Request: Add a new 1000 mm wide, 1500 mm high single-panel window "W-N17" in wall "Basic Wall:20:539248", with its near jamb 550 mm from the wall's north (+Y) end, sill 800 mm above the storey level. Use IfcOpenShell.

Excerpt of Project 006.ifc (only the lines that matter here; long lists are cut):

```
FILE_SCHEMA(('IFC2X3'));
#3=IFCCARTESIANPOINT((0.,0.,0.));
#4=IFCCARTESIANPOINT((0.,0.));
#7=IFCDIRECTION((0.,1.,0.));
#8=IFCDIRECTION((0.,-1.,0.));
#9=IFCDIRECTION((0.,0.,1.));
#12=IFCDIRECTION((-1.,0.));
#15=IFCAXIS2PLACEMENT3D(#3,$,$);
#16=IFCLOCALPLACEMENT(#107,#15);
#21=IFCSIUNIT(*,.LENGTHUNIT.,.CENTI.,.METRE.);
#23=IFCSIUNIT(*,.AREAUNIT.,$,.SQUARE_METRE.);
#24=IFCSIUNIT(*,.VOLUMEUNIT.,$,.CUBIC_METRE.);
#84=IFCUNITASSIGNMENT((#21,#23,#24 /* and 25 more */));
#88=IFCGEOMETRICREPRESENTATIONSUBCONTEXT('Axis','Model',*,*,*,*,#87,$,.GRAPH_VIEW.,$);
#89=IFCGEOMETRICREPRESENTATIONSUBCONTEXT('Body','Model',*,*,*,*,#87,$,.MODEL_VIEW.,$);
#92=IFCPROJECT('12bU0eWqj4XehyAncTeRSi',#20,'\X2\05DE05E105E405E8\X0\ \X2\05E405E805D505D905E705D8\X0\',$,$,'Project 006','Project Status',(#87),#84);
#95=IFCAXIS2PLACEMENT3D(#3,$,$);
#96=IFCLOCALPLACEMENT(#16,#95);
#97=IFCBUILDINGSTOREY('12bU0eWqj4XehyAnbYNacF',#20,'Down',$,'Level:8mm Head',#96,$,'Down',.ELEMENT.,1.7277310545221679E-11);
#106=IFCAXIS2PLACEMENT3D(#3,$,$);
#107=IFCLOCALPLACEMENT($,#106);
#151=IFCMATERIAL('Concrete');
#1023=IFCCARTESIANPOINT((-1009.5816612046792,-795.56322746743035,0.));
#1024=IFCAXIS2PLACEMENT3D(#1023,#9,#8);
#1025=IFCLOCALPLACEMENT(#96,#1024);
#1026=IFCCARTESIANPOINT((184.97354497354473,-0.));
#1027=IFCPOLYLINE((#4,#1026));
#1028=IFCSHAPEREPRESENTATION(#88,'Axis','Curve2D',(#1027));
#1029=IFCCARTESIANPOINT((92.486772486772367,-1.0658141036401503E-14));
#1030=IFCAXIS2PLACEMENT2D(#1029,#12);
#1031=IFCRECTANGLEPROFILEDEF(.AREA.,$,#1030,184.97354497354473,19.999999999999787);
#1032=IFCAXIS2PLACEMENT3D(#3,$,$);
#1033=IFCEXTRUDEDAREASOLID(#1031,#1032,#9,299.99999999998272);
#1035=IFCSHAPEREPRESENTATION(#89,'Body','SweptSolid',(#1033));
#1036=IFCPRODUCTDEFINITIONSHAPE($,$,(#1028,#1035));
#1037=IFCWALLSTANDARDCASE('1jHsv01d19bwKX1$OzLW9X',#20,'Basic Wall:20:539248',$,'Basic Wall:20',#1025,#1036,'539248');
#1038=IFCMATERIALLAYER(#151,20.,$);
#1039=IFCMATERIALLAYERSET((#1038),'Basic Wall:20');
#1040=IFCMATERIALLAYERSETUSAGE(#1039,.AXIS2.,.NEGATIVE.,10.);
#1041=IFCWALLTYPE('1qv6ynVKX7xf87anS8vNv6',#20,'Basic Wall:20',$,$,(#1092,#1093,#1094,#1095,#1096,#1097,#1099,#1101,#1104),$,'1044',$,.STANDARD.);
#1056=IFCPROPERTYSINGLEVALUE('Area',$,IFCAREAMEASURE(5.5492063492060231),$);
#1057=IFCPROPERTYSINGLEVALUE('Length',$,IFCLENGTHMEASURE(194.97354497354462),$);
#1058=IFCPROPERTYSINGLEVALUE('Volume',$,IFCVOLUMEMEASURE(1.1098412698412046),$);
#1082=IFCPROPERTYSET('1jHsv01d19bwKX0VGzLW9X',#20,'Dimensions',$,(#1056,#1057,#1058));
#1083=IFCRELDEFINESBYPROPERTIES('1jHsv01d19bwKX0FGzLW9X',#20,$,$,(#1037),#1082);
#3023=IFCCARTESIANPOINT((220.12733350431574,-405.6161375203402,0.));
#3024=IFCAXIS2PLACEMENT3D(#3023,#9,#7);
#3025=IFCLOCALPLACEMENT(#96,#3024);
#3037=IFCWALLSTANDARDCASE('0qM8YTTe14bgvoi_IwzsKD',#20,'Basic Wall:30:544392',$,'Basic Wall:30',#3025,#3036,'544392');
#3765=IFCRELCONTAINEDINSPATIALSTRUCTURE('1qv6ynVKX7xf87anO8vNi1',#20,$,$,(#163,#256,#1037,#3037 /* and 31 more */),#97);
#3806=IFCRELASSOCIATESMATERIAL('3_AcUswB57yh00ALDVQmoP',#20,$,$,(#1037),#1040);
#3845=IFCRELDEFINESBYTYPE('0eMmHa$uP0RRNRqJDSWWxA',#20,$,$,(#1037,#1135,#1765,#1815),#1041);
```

```python
import numpy as np
import ifcopenshell
import ifcopenshell.api.feature
import ifcopenshell.api.geometry
import ifcopenshell.api.pset
import ifcopenshell.api.root
import ifcopenshell.api.spatial
import ifcopenshell.api.type
import ifcopenshell.geom
import ifcopenshell.util.element
import ifcopenshell.util.placement
import ifcopenshell.util.representation
import ifcopenshell.util.shape
import ifcopenshell.util.unit

model = ifcopenshell.open("Project 006.ifc")
unit_scale = ifcopenshell.util.unit.calculate_unit_scale(model)
area_scale = ifcopenshell.util.unit.calculate_unit_scale(model, "AREAUNIT")
volume_scale = ifcopenshell.util.unit.calculate_unit_scale(model, "VOLUMEUNIT")
settings = ifcopenshell.geom.settings()


def volume(element):
    """Net volume in cubic metres, openings subtracted."""
    shape = ifcopenshell.geom.create_shape(settings, element)
    return ifcopenshell.util.shape.get_volume(shape.geometry)


wall = model.by_guid("1jHsv01d19bwKX1$OzLW9X")
storey = ifcopenshell.util.element.get_container(wall, ifc_class="IfcBuildingStorey")
context = ifcopenshell.util.representation.get_context(model, "Model", "Body", "MODEL_VIEW")
before = volume(wall)

width, height, from_end, sill = 1, 1.5, 0.55, 0.8  # metres

# The wall runs along its own X axis, and the end named is its -X end.
wall_shape = ifcopenshell.geom.create_shape(settings, wall)
x, y, z = ifcopenshell.util.shape.get_vertices(wall_shape.geometry).T
start = x.min() + from_end
face, thickness = float(y.min()), float(y.max() - y.min())
wall_matrix = ifcopenshell.util.placement.get_local_placement(wall.ObjectPlacement)
level = ifcopenshell.util.placement.get_local_placement(storey.ObjectPlacement)[2, 3]


def in_wall(x, y):
    """Placement at x, y metres in the wall's axes, at sill height."""
    matrix = wall_matrix.copy()
    matrix[:, 3] = wall_matrix @ np.array([x / unit_scale, y / unit_scale, 0.0, 1.0])
    matrix[2, 3] = level + sill / unit_scale
    return matrix


# Opening: a box that overshoots both wall faces by 50 mm.
opening = ifcopenshell.api.root.create_entity(model, ifc_class="IfcOpeningElement")
box = ifcopenshell.api.geometry.add_wall_representation(
    model, context=context, length=width, height=height, thickness=thickness + 0.1
)
ifcopenshell.api.geometry.assign_representation(model, product=opening, representation=box)
ifcopenshell.api.geometry.edit_object_placement(model, product=opening, matrix=in_wall(start, face - 0.05), is_si=False)
ifcopenshell.api.feature.add_feature(model, feature=opening, element=wall)

window = ifcopenshell.api.root.create_entity(model, ifc_class="IfcWindow", name="W-N17")
window.OverallWidth, window.OverallHeight = width / unit_scale, height / unit_scale
body = ifcopenshell.api.geometry.add_window_representation(
    model,
    context=context,
    overall_width=window.OverallWidth,
    overall_height=window.OverallHeight,
    partition_type="SINGLE_PANEL",
)
ifcopenshell.api.geometry.assign_representation(model, product=window, representation=body)
ifcopenshell.api.spatial.assign_container(model, products=[window], relating_structure=storey)
fills = ifcopenshell.api.feature.add_filling(model, opening=opening, element=window)
fills.OwnerHistory = window.OwnerHistory  # required in IFC2X3

# IFC2X3 keeps the operation on the window style.
style = ifcopenshell.api.root.create_entity(model, ifc_class="IfcWindowStyle", name="W-N17")
style.OperationType, style.ConstructionType = "SINGLE_PANEL", "NOTDEFINED"
style.ParameterTakesPrecedence = style.Sizeable = False
ifcopenshell.api.type.assign_type(model, related_objects=[window], relating_type=style)

# Centre the window in the wall's thickness.
ifcopenshell.api.geometry.edit_object_placement(model, product=window, matrix=in_wall(start, face), is_si=False)
window_shape = ifcopenshell.geom.create_shape(settings, window)
depth = ifcopenshell.util.shape.get_vertices(window_shape.geometry)[:, 1]
offset = face + thickness / 2 - (depth.min() + depth.max()) / 2
ifcopenshell.api.geometry.edit_object_placement(model, product=window, matrix=in_wall(start, offset), is_si=False)

after = volume(wall)

# Update the wall's stored quantities.
pset = model.by_id(ifcopenshell.util.element.get_pset(wall, "Dimensions", should_inherit=False)["id"])
ifcopenshell.api.pset.edit_pset(model, pset=pset, properties={
    "Area": model.create_entity("IfcAreaMeasure", after / thickness / area_scale),
    "Volume": model.create_entity("IfcVolumeMeasure", after / volume_scale),
})

print(f"wall volume {before:.3f} -> {after:.3f} m3")

model.write("Project 006-out.ifc")
```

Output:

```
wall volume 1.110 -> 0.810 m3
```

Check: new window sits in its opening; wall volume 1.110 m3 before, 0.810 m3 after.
